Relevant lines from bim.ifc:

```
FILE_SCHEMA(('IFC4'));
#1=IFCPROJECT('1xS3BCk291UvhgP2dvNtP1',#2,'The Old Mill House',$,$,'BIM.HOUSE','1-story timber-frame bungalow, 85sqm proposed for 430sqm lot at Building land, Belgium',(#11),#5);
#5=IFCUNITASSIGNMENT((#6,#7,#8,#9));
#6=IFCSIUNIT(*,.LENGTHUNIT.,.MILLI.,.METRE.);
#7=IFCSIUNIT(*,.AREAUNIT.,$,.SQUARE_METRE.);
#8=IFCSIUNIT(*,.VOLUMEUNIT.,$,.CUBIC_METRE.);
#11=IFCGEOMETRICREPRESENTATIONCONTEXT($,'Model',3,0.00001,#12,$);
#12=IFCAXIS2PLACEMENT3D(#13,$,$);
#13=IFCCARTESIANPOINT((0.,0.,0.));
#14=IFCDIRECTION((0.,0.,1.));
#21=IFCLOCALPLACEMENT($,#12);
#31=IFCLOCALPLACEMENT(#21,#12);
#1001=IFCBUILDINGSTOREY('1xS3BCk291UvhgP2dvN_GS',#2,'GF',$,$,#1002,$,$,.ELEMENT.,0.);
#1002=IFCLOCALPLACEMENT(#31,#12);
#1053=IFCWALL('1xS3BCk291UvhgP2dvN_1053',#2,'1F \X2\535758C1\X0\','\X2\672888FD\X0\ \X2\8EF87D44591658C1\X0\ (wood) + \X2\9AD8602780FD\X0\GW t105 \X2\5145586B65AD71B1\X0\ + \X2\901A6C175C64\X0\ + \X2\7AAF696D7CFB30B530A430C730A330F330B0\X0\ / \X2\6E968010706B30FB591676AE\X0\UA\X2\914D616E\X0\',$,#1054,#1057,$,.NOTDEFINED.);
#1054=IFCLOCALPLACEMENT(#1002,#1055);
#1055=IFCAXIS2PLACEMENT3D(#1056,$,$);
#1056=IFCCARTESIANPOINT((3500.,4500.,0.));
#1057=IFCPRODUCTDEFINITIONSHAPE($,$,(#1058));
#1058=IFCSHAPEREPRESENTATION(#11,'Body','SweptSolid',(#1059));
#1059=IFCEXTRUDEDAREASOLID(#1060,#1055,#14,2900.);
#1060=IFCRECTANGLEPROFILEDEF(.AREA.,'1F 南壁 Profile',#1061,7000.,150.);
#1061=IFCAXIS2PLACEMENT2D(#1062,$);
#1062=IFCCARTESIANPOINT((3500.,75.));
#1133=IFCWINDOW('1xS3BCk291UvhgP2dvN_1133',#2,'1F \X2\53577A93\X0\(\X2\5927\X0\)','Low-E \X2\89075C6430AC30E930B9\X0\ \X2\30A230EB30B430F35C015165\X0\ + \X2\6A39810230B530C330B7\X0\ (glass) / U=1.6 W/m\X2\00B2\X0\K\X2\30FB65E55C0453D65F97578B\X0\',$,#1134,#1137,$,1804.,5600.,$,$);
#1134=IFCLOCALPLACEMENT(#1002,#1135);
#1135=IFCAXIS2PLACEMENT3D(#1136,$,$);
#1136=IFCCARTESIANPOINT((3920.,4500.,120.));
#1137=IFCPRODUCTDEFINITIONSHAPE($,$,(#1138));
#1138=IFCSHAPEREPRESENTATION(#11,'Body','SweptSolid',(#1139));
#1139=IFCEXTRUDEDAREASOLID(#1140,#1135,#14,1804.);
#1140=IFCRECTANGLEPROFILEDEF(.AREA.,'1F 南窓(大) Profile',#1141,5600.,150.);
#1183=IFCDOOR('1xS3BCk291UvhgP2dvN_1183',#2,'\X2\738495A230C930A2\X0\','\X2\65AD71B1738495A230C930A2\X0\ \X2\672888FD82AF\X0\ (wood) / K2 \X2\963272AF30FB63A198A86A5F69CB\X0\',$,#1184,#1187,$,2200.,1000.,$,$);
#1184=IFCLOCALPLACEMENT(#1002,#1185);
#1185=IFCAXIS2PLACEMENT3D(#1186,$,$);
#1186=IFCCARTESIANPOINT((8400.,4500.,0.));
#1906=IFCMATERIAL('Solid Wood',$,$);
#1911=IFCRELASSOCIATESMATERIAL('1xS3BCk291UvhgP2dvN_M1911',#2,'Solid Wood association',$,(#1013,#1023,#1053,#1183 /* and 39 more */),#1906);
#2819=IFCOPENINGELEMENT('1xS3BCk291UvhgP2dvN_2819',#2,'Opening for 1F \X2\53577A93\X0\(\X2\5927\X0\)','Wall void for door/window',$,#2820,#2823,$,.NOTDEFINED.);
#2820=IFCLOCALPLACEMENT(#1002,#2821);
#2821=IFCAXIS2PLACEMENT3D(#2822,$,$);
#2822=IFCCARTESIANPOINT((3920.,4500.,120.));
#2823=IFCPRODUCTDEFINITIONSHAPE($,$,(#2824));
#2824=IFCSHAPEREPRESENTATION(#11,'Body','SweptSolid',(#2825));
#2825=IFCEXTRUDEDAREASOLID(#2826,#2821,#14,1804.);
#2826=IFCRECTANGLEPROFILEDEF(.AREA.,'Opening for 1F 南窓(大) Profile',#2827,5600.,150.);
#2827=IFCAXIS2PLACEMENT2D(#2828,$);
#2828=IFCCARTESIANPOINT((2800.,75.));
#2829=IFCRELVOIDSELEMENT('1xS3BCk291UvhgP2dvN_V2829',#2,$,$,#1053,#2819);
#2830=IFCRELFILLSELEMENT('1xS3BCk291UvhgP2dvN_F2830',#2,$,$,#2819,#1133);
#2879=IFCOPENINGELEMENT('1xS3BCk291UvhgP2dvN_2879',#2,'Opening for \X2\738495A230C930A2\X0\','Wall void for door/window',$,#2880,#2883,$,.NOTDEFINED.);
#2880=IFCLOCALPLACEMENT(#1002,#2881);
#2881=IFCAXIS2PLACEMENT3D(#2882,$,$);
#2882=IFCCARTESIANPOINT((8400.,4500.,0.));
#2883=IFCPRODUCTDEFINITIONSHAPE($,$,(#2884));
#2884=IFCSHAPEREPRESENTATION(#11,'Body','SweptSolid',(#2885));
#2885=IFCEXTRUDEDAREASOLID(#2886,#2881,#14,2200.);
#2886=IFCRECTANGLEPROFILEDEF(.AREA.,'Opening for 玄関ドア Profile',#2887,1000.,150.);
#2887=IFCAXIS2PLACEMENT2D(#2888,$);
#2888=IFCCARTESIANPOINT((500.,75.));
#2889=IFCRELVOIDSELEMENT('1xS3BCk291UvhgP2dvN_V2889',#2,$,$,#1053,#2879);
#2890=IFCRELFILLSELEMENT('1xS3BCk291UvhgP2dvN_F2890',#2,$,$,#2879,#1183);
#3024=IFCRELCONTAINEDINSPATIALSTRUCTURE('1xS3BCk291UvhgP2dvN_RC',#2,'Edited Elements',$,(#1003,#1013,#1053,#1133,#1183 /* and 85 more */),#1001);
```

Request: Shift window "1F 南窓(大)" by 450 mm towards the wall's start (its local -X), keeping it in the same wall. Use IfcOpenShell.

```python
import ifcopenshell
import ifcopenshell.api.geometry
import ifcopenshell.util.placement
import ifcopenshell.util.unit

model = ifcopenshell.open("bim.ifc")
unit_scale = ifcopenshell.util.unit.calculate_unit_scale(model)

window = model.by_guid("1xS3BCk291UvhgP2dvN_1133")
opening = window.FillsVoids[0].RelatingOpeningElement
wall = opening.VoidsElements[0].RelatingBuildingElement

wall_matrix = ifcopenshell.util.placement.get_local_placement(wall.ObjectPlacement)
shift = wall_matrix[:3, 0] * -0.45 / unit_scale
before = ifcopenshell.util.placement.get_local_placement(window.ObjectPlacement)[:3, 3].copy()

# The window is not placed relative to its opening, so move both.
for product in (opening, window):
    matrix = ifcopenshell.util.placement.get_local_placement(product.ObjectPlacement)
    matrix[:3, 3] += shift
    ifcopenshell.api.geometry.edit_object_placement(model, product=product, matrix=matrix, is_si=False)

after = ifcopenshell.util.placement.get_local_placement(window.ObjectPlacement)[:3, 3]
print("window moved by", (after - before).round(3) + 0.0)

model.write("bim_v2.ifc")
```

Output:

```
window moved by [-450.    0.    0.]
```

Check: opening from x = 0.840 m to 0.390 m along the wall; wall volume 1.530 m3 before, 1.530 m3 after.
